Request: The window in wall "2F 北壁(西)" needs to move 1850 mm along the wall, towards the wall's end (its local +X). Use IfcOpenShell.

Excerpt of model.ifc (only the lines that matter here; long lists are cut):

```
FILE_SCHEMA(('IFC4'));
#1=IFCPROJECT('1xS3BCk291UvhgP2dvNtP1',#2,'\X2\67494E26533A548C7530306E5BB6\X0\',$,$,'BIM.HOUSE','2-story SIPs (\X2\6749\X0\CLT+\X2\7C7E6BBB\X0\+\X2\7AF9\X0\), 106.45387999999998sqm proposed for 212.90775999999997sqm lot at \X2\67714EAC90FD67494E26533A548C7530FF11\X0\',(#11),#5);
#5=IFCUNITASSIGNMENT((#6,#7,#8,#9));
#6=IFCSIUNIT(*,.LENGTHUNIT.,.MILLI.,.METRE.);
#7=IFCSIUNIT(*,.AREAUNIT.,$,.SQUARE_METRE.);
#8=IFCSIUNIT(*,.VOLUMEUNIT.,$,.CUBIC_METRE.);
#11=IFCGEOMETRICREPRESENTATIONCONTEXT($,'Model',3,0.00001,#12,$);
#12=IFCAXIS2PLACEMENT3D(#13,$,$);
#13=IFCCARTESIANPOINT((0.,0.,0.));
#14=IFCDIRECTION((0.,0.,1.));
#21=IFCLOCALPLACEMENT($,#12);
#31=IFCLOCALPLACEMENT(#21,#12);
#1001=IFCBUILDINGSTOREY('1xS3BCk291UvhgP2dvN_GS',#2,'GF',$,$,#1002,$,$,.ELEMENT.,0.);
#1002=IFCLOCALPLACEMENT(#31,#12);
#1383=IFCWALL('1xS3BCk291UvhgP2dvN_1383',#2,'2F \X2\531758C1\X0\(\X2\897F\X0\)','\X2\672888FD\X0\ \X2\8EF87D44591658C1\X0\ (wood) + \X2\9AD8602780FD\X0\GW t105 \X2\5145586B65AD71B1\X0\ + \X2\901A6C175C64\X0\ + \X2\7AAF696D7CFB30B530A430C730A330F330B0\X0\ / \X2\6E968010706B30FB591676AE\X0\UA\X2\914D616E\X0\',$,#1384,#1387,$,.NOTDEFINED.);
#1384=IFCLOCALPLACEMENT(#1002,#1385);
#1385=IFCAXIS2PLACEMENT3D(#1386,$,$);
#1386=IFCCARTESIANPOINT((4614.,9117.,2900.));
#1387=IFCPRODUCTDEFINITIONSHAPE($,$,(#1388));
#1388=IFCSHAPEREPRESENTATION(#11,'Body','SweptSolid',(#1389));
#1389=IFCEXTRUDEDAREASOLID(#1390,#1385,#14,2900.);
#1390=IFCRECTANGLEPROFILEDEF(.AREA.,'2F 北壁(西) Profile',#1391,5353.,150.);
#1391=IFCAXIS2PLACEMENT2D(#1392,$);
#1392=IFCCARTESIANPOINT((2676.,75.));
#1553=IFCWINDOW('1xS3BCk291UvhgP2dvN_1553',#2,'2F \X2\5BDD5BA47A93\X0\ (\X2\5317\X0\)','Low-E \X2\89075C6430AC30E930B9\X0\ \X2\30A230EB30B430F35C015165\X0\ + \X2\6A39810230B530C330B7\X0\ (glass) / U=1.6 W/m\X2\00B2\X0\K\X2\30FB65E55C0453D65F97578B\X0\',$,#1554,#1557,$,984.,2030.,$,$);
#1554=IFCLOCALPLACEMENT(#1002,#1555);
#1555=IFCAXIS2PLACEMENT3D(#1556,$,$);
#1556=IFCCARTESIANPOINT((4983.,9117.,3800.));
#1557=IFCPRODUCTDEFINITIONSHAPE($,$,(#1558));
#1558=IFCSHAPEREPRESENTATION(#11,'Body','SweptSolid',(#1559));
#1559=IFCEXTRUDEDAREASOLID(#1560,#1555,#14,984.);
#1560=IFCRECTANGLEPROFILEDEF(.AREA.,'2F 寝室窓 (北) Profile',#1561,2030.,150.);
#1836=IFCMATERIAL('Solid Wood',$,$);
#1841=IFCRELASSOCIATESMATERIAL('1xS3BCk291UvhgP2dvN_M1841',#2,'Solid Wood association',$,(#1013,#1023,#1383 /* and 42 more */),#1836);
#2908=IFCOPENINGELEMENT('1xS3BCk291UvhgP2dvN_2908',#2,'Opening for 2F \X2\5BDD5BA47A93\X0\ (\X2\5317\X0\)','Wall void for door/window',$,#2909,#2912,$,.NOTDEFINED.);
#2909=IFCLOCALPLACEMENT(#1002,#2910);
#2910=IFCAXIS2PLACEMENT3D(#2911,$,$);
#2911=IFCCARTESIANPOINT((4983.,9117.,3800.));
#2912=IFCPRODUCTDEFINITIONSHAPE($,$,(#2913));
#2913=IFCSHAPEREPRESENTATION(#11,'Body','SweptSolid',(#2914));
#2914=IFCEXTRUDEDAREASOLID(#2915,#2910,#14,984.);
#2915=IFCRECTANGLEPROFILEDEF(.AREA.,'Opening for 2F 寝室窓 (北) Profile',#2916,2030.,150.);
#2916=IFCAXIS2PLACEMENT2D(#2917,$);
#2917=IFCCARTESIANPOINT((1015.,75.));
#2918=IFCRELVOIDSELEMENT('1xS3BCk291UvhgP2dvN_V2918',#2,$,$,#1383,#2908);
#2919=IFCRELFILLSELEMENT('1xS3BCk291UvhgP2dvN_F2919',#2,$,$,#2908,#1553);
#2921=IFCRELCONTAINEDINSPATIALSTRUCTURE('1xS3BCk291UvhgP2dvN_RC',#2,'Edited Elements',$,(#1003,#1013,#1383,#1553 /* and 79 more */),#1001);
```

```python
import ifcopenshell
import ifcopenshell.api.geometry
import ifcopenshell.util.placement
import ifcopenshell.util.unit

model = ifcopenshell.open("model.ifc")
unit_scale = ifcopenshell.util.unit.calculate_unit_scale(model)

window = model.by_guid("1xS3BCk291UvhgP2dvN_1553")
opening = window.FillsVoids[0].RelatingOpeningElement
wall = opening.VoidsElements[0].RelatingBuildingElement

wall_matrix = ifcopenshell.util.placement.get_local_placement(wall.ObjectPlacement)
shift = wall_matrix[:3, 0] * 1.85 / unit_scale
before = ifcopenshell.util.placement.get_local_placement(window.ObjectPlacement)[:3, 3].copy()

# The window is not placed relative to its opening, so move both.
for product in (opening, window):
    matrix = ifcopenshell.util.placement.get_local_placement(product.ObjectPlacement)
    matrix[:3, 3] += shift
    ifcopenshell.api.geometry.edit_object_placement(model, product=product, matrix=matrix, is_si=False)

after = ifcopenshell.util.placement.get_local_placement(window.ObjectPlacement)[:3, 3]
print("window moved by", (after - before).round(3) + 0.0)

model.write("model-out.ifc")
```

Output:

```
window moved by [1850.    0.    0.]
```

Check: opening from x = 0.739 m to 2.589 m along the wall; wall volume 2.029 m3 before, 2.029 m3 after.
